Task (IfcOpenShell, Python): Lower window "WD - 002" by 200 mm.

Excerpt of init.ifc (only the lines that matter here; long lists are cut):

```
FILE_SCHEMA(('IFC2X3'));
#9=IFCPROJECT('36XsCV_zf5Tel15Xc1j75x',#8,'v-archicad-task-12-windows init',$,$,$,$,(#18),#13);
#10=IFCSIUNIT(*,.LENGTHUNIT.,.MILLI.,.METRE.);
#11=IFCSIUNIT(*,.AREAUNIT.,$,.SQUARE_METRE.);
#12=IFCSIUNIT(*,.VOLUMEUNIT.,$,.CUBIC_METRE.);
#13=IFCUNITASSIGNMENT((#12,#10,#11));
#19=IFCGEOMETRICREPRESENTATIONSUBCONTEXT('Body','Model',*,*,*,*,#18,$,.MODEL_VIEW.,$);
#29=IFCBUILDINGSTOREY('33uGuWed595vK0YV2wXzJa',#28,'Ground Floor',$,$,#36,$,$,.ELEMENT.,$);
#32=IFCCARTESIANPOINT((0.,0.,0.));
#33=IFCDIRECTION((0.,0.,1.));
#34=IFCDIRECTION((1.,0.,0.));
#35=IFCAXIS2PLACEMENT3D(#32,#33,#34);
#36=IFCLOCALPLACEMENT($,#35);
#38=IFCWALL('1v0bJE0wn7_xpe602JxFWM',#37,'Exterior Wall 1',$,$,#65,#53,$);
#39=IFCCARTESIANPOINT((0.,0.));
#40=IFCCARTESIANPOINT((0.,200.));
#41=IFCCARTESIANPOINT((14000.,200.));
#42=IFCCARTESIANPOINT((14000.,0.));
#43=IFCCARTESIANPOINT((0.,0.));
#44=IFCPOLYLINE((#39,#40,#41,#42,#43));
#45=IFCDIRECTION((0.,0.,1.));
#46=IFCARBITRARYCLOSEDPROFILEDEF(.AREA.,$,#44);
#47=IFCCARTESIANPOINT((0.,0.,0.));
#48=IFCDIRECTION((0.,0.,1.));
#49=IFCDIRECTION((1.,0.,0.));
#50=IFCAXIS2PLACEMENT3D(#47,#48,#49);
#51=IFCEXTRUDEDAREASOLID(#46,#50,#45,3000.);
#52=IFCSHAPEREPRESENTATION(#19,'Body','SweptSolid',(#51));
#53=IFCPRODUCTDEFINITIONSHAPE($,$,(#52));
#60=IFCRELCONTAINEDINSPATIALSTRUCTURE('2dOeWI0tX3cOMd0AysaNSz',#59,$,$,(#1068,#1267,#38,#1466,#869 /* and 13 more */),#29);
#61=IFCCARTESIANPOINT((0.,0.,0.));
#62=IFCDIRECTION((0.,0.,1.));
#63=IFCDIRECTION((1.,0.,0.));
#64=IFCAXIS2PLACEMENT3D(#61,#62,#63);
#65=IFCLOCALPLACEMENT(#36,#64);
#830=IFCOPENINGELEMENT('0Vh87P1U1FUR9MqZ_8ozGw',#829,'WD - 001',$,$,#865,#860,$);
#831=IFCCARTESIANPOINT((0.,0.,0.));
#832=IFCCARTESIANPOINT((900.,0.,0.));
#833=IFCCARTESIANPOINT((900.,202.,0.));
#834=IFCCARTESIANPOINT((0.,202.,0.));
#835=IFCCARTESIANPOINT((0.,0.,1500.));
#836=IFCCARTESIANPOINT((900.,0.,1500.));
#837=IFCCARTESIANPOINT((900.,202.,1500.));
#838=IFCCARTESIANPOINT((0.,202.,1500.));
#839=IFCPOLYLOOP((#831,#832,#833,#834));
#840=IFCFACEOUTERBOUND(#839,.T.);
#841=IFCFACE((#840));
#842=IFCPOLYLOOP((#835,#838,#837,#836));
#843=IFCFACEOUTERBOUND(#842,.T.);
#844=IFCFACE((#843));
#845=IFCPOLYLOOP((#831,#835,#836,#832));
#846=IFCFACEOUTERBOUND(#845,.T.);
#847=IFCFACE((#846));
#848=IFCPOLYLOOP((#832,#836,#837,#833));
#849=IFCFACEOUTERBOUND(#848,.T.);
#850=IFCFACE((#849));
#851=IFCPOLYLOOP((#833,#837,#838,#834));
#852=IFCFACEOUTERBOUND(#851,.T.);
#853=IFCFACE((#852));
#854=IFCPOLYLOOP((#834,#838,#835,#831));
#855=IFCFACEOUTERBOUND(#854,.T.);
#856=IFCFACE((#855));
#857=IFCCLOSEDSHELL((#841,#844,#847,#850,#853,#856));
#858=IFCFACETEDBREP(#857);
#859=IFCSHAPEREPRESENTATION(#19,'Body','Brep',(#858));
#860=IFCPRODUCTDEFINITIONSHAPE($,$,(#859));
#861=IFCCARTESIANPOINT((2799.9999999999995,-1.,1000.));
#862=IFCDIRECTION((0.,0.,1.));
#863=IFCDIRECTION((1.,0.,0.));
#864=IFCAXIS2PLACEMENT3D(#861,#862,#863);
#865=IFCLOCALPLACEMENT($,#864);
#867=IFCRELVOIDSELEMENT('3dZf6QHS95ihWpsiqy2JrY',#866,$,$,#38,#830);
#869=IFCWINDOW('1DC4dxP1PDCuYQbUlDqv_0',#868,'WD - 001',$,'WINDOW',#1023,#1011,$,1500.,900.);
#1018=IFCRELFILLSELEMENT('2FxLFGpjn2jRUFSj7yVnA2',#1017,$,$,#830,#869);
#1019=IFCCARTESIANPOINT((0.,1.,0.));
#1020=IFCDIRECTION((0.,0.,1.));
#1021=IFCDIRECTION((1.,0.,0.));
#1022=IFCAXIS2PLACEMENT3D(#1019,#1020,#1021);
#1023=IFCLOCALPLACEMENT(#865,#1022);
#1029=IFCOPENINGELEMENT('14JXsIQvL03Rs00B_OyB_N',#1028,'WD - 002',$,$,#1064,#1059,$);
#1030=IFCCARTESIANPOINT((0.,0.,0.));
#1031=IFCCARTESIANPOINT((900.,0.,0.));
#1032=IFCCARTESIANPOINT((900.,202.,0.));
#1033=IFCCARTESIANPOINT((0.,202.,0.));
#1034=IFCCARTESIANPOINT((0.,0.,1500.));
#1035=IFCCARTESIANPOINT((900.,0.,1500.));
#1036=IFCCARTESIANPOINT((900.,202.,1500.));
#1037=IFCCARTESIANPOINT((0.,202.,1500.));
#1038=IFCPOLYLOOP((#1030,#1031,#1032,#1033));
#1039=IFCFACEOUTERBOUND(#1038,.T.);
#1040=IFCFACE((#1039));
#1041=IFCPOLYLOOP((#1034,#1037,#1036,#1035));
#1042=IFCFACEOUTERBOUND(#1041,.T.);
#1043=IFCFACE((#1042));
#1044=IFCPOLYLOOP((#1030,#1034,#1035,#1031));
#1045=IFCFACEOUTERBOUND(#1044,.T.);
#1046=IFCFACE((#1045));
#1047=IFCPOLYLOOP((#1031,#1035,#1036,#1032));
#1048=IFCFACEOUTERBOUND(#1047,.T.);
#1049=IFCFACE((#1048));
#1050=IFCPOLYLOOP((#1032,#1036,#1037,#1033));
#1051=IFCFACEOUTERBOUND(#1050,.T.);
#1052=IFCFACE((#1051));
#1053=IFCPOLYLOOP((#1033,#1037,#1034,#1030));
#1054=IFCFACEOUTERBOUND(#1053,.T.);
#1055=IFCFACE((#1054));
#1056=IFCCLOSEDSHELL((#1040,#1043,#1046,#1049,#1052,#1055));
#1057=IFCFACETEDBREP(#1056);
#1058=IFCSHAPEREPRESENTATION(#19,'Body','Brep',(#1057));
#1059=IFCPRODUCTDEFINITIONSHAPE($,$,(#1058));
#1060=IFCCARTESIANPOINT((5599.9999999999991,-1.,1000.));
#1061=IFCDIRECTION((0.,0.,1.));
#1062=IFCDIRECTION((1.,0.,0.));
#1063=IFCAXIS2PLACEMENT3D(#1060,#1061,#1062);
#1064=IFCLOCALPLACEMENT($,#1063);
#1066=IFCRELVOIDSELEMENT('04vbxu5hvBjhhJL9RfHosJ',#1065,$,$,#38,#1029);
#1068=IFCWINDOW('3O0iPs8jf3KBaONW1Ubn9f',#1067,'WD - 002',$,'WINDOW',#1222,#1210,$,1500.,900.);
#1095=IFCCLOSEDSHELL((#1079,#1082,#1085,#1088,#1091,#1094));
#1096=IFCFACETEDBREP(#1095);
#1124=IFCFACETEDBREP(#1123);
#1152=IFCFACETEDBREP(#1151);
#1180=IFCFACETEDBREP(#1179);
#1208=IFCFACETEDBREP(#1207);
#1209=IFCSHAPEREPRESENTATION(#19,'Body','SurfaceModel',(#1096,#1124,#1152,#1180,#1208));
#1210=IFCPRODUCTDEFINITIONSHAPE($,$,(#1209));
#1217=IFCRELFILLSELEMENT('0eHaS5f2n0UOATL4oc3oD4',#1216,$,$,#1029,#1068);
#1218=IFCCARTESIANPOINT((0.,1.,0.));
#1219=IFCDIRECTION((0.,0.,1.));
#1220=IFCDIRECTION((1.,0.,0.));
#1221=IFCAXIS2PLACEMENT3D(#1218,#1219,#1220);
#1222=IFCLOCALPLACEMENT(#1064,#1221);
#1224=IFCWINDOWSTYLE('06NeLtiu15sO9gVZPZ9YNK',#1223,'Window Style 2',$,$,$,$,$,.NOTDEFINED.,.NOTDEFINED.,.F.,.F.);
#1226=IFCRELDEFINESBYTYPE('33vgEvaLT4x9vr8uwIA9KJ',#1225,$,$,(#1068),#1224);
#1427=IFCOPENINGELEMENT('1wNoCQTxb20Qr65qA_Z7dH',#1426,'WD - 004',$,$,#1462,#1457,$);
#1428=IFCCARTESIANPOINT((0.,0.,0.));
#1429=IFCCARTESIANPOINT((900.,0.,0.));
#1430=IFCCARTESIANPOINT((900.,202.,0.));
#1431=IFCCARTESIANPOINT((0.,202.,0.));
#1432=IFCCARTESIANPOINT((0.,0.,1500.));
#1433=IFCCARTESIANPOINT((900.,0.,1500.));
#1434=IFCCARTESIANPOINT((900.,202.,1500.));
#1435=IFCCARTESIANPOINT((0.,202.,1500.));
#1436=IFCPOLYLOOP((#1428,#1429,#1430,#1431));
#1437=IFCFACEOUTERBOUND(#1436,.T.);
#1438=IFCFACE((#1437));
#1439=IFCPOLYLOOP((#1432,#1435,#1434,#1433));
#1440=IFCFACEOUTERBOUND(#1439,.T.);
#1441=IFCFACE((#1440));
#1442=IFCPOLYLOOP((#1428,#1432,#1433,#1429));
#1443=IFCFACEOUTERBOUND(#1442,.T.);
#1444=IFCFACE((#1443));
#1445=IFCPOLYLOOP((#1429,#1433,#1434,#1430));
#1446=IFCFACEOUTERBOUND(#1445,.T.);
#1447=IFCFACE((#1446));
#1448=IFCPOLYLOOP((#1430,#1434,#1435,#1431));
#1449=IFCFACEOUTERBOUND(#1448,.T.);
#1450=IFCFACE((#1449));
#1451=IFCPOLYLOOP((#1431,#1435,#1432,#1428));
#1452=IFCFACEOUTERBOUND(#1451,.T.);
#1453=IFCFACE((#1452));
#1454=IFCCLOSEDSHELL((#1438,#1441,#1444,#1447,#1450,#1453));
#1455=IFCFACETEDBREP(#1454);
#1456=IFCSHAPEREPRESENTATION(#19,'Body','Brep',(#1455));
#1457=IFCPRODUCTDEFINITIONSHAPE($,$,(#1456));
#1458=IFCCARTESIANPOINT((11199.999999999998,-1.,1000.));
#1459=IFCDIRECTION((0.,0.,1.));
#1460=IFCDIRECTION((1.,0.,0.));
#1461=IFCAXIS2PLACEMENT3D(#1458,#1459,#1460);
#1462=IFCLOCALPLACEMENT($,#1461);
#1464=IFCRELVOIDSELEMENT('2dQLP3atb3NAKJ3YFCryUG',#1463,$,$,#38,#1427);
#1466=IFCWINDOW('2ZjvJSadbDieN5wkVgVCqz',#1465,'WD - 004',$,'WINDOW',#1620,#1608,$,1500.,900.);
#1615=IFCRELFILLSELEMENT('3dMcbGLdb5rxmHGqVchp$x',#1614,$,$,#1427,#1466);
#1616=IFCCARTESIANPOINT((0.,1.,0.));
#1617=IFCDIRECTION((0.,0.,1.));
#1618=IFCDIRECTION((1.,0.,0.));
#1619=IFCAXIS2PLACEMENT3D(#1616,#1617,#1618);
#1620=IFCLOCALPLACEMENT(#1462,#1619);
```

```python
import numpy as np
import ifcopenshell
import ifcopenshell.api.geometry
import ifcopenshell.util.placement
import ifcopenshell.util.unit

model = ifcopenshell.open("init.ifc")
unit_scale = ifcopenshell.util.unit.calculate_unit_scale(model)

window = model.by_guid("3O0iPs8jf3KBaONW1Ubn9f")
opening = window.FillsVoids[0].RelatingOpeningElement
dz = -0.2 / unit_scale

shift = np.array([0.0, 0.0, dz])
# The window is placed relative to its opening, so it follows when the opening moves.
matrix = ifcopenshell.util.placement.get_local_placement(opening.ObjectPlacement)
matrix[:3, 3] += shift
ifcopenshell.api.geometry.edit_object_placement(
    model, product=opening, matrix=matrix, is_si=False, should_transform_children=True
)

print(f"moved by {dz * unit_scale:+.3f} m")

model.write("init_rev.ifc")
```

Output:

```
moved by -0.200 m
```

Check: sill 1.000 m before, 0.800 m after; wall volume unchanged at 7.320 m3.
